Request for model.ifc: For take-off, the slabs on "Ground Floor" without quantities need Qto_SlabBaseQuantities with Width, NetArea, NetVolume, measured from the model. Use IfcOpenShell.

First a look at what the model holds.

```python
import ifcopenshell
import ifcopenshell.util.element
import ifcopenshell.util.unit

model = ifcopenshell.open("model.ifc")
print(model.schema)
for unit_type in ("LENGTHUNIT", "AREAUNIT", "VOLUMEUNIT"):
    print(unit_type, ifcopenshell.util.unit.calculate_unit_scale(model, unit_type))
storey = next(s for s in model.by_type("IfcBuildingStorey") if s.Name == "Ground Floor")
slabs = [e for e in ifcopenshell.util.element.get_decomposition(storey) if e.is_a("IfcSlab")]
for e in sorted(slabs, key=lambda e: e.id()):
    print(e.id(), e.is_a(), e.Name, list(ifcopenshell.util.element.get_psets(e, qtos_only=True)), sep=" | ")
```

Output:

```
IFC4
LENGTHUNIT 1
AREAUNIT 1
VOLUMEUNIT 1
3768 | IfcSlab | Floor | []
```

```python
import ifcopenshell
import ifcopenshell.api.pset
import ifcopenshell.geom
import ifcopenshell.util.element
import ifcopenshell.util.shape
import ifcopenshell.util.unit

model = ifcopenshell.open("model.ifc")
unit_scale = ifcopenshell.util.unit.calculate_unit_scale(model)
area_scale = ifcopenshell.util.unit.calculate_unit_scale(model, "AREAUNIT")
volume_scale = ifcopenshell.util.unit.calculate_unit_scale(model, "VOLUMEUNIT")
settings = ifcopenshell.geom.settings()

storey = next(s for s in model.by_type("IfcBuildingStorey") if s.Name == "Ground Floor")
slabs = [e for e in ifcopenshell.util.element.get_decomposition(storey) if e.is_a("IfcSlab")]

for e in sorted(slabs, key=lambda e: e.id()):
    if ifcopenshell.util.element.get_psets(e, qtos_only=True, should_inherit=False):
        continue
    # Geometry comes back in metres, in the element's own axes.
    shape = ifcopenshell.geom.create_shape(settings, e)
    values = {
        "Width": ifcopenshell.util.shape.get_z(shape.geometry) / unit_scale,
        "NetArea": ifcopenshell.util.shape.get_footprint_area(shape.geometry) / area_scale,
        "NetVolume": ifcopenshell.util.shape.get_volume(shape.geometry) / volume_scale,
    }
    qto = ifcopenshell.api.pset.add_qto(model, product=e, name="Qto_SlabBaseQuantities")
    ifcopenshell.api.pset.edit_qto(model, qto=qto, properties=values)
    print(e.id(), {k: round(v, 3) for k, v in values.items()})

model.write("model_updated.ifc")
```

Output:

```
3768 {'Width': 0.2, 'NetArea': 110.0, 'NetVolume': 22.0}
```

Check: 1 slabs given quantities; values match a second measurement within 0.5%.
